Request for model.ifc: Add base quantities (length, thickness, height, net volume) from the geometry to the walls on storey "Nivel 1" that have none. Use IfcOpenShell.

First a look at what the model holds.

```python
import ifcopenshell
import ifcopenshell.util.element
import ifcopenshell.util.unit

model = ifcopenshell.open("model.ifc")
print(model.schema)
for unit_type in ("LENGTHUNIT", "AREAUNIT", "VOLUMEUNIT"):
    print(unit_type, ifcopenshell.util.unit.calculate_unit_scale(model, unit_type))
storey = next(s for s in model.by_type("IfcBuildingStorey") if s.Name == "Nivel 1")
walls = [e for e in ifcopenshell.util.element.get_decomposition(storey) if e.is_a("IfcWall")]
for e in sorted(walls, key=lambda e: e.id()):
    print(e.id(), e.is_a(), e.Name, list(ifcopenshell.util.element.get_psets(e, qtos_only=True)), sep=" | ")
```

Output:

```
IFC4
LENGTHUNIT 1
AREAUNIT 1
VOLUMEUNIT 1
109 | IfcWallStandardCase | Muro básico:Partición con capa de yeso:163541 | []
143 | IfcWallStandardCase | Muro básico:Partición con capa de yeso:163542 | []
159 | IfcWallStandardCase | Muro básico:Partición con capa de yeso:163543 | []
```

```python
import ifcopenshell
import ifcopenshell.api.pset
import ifcopenshell.geom
import ifcopenshell.util.element
import ifcopenshell.util.shape
import ifcopenshell.util.unit

model = ifcopenshell.open("model.ifc")
unit_scale = ifcopenshell.util.unit.calculate_unit_scale(model)
volume_scale = ifcopenshell.util.unit.calculate_unit_scale(model, "VOLUMEUNIT")
settings = ifcopenshell.geom.settings()

storey = next(s for s in model.by_type("IfcBuildingStorey") if s.Name == "Nivel 1")
walls = [e for e in ifcopenshell.util.element.get_decomposition(storey) if e.is_a("IfcWall")]

for e in sorted(walls, key=lambda e: e.id()):
    if ifcopenshell.util.element.get_psets(e, qtos_only=True, should_inherit=False):
        continue
    # Geometry comes back in metres, in the element's own axes.
    shape = ifcopenshell.geom.create_shape(settings, e)
    values = {
        "Length": ifcopenshell.util.shape.get_x(shape.geometry) / unit_scale,
        "Width": ifcopenshell.util.shape.get_y(shape.geometry) / unit_scale,
        "Height": ifcopenshell.util.shape.get_z(shape.geometry) / unit_scale,
        "NetVolume": ifcopenshell.util.shape.get_volume(shape.geometry) / volume_scale,
    }
    qto = ifcopenshell.api.pset.add_qto(model, product=e, name="Qto_WallBaseQuantities")
    ifcopenshell.api.pset.edit_qto(model, qto=qto, properties=values)
    print(e.id(), {k: round(v, 3) for k, v in values.items()})

model.write("model_edited.ifc")
```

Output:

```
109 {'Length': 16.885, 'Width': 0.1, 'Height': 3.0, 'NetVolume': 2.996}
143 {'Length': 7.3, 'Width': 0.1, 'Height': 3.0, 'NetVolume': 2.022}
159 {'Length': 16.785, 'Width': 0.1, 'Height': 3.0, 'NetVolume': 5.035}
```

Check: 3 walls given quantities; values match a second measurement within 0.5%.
